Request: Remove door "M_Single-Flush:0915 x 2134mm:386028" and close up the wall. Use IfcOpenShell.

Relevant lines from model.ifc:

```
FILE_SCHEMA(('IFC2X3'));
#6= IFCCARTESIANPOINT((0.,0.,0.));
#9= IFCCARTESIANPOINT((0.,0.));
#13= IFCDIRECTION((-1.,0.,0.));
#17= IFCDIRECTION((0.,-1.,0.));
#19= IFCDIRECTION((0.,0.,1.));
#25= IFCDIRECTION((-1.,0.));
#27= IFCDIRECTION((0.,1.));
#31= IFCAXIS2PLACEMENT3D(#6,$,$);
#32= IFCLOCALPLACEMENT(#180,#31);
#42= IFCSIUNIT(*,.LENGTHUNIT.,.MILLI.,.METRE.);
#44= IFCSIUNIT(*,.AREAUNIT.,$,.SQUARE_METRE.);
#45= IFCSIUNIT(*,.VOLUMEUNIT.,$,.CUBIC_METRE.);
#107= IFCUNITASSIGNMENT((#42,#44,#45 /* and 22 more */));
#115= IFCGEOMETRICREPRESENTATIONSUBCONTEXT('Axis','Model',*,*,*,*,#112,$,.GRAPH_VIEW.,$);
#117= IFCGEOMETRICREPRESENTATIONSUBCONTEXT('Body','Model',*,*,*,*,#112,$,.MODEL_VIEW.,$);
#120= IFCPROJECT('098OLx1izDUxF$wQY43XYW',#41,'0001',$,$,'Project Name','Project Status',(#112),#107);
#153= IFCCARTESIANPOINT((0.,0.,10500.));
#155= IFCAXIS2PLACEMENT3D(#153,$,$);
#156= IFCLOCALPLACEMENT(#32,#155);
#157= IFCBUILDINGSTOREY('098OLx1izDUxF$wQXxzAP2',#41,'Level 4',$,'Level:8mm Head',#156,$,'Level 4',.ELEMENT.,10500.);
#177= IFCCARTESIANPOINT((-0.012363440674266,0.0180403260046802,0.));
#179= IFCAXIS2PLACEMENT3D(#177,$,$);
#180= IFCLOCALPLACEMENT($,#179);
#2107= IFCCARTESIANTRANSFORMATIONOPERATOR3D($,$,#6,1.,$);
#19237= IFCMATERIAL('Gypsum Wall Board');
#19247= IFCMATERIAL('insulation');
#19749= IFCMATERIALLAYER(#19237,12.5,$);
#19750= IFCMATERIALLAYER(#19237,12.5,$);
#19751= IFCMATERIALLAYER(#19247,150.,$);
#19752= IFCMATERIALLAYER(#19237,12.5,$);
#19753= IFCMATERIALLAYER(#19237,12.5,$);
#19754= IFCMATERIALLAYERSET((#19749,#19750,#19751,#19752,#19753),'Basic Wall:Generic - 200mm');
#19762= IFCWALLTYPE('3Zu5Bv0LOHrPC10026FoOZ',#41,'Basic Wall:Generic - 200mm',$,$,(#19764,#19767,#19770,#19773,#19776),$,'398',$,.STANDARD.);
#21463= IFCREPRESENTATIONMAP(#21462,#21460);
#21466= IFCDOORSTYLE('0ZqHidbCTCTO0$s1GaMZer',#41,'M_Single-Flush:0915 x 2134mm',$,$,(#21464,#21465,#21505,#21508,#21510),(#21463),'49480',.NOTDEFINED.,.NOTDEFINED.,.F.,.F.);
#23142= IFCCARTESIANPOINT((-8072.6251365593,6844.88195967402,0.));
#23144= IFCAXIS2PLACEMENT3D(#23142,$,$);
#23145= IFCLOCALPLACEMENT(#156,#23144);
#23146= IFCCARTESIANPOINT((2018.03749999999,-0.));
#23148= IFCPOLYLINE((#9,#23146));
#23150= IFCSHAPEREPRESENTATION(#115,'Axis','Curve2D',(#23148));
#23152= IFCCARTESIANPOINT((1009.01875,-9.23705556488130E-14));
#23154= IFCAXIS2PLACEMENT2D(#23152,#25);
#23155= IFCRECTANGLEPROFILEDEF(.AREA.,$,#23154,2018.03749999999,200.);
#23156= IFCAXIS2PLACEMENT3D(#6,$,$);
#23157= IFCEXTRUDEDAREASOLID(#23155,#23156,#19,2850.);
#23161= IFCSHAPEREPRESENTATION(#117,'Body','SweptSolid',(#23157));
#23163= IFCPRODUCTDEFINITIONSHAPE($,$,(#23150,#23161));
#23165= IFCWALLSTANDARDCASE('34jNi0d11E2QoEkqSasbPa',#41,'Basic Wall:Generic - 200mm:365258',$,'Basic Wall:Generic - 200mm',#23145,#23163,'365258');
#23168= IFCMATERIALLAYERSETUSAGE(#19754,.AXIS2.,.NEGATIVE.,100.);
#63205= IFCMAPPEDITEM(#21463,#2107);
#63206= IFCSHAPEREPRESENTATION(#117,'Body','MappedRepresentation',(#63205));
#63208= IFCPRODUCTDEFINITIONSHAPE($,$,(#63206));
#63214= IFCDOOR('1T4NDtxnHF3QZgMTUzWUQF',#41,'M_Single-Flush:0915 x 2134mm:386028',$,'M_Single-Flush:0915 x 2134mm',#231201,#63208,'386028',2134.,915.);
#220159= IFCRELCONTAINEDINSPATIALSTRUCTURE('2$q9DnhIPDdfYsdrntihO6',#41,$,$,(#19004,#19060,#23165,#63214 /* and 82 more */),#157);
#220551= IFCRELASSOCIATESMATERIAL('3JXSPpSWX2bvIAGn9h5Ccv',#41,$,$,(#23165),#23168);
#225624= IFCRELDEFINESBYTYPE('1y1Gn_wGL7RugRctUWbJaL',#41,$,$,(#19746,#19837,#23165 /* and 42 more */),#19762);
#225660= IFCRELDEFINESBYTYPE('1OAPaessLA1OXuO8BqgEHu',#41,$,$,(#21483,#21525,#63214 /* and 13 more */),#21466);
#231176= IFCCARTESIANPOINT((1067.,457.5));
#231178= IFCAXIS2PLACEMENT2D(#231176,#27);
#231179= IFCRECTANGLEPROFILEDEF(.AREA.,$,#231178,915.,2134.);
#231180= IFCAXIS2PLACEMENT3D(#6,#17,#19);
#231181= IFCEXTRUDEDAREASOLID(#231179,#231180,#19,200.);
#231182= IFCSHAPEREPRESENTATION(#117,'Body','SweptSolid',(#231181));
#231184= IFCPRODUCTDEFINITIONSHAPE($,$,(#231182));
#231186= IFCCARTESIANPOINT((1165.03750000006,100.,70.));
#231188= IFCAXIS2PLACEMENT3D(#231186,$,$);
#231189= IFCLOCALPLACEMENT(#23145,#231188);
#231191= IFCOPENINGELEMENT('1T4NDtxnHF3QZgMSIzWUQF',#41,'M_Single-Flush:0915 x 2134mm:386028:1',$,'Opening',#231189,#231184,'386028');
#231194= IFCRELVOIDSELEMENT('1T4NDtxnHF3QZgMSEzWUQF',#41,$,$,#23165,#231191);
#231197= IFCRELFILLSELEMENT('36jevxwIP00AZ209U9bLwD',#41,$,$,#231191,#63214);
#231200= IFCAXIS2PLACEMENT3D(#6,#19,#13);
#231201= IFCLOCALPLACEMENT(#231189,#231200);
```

```python
import ifcopenshell
import ifcopenshell.api.feature
import ifcopenshell.api.root
import ifcopenshell.geom
import ifcopenshell.util.shape

model = ifcopenshell.open("model.ifc")
settings = ifcopenshell.geom.settings()


def volume(element):
    """Net volume in cubic metres, openings subtracted."""
    shape = ifcopenshell.geom.create_shape(settings, element)
    return ifcopenshell.util.shape.get_volume(shape.geometry)


door = model.by_guid("1T4NDtxnHF3QZgMTUzWUQF")
opening = door.FillsVoids[0].RelatingOpeningElement
wall = opening.VoidsElements[0].RelatingBuildingElement
before = volume(wall)

ifcopenshell.api.root.remove_product(model, product=door)
ifcopenshell.api.feature.remove_feature(model, feature=opening)

after = volume(wall)

print(f"wall volume {before:.3f} -> {after:.3f} m3")

model.write("model-out.ifc")
```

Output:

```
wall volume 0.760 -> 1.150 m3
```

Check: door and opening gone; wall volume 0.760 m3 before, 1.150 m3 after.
